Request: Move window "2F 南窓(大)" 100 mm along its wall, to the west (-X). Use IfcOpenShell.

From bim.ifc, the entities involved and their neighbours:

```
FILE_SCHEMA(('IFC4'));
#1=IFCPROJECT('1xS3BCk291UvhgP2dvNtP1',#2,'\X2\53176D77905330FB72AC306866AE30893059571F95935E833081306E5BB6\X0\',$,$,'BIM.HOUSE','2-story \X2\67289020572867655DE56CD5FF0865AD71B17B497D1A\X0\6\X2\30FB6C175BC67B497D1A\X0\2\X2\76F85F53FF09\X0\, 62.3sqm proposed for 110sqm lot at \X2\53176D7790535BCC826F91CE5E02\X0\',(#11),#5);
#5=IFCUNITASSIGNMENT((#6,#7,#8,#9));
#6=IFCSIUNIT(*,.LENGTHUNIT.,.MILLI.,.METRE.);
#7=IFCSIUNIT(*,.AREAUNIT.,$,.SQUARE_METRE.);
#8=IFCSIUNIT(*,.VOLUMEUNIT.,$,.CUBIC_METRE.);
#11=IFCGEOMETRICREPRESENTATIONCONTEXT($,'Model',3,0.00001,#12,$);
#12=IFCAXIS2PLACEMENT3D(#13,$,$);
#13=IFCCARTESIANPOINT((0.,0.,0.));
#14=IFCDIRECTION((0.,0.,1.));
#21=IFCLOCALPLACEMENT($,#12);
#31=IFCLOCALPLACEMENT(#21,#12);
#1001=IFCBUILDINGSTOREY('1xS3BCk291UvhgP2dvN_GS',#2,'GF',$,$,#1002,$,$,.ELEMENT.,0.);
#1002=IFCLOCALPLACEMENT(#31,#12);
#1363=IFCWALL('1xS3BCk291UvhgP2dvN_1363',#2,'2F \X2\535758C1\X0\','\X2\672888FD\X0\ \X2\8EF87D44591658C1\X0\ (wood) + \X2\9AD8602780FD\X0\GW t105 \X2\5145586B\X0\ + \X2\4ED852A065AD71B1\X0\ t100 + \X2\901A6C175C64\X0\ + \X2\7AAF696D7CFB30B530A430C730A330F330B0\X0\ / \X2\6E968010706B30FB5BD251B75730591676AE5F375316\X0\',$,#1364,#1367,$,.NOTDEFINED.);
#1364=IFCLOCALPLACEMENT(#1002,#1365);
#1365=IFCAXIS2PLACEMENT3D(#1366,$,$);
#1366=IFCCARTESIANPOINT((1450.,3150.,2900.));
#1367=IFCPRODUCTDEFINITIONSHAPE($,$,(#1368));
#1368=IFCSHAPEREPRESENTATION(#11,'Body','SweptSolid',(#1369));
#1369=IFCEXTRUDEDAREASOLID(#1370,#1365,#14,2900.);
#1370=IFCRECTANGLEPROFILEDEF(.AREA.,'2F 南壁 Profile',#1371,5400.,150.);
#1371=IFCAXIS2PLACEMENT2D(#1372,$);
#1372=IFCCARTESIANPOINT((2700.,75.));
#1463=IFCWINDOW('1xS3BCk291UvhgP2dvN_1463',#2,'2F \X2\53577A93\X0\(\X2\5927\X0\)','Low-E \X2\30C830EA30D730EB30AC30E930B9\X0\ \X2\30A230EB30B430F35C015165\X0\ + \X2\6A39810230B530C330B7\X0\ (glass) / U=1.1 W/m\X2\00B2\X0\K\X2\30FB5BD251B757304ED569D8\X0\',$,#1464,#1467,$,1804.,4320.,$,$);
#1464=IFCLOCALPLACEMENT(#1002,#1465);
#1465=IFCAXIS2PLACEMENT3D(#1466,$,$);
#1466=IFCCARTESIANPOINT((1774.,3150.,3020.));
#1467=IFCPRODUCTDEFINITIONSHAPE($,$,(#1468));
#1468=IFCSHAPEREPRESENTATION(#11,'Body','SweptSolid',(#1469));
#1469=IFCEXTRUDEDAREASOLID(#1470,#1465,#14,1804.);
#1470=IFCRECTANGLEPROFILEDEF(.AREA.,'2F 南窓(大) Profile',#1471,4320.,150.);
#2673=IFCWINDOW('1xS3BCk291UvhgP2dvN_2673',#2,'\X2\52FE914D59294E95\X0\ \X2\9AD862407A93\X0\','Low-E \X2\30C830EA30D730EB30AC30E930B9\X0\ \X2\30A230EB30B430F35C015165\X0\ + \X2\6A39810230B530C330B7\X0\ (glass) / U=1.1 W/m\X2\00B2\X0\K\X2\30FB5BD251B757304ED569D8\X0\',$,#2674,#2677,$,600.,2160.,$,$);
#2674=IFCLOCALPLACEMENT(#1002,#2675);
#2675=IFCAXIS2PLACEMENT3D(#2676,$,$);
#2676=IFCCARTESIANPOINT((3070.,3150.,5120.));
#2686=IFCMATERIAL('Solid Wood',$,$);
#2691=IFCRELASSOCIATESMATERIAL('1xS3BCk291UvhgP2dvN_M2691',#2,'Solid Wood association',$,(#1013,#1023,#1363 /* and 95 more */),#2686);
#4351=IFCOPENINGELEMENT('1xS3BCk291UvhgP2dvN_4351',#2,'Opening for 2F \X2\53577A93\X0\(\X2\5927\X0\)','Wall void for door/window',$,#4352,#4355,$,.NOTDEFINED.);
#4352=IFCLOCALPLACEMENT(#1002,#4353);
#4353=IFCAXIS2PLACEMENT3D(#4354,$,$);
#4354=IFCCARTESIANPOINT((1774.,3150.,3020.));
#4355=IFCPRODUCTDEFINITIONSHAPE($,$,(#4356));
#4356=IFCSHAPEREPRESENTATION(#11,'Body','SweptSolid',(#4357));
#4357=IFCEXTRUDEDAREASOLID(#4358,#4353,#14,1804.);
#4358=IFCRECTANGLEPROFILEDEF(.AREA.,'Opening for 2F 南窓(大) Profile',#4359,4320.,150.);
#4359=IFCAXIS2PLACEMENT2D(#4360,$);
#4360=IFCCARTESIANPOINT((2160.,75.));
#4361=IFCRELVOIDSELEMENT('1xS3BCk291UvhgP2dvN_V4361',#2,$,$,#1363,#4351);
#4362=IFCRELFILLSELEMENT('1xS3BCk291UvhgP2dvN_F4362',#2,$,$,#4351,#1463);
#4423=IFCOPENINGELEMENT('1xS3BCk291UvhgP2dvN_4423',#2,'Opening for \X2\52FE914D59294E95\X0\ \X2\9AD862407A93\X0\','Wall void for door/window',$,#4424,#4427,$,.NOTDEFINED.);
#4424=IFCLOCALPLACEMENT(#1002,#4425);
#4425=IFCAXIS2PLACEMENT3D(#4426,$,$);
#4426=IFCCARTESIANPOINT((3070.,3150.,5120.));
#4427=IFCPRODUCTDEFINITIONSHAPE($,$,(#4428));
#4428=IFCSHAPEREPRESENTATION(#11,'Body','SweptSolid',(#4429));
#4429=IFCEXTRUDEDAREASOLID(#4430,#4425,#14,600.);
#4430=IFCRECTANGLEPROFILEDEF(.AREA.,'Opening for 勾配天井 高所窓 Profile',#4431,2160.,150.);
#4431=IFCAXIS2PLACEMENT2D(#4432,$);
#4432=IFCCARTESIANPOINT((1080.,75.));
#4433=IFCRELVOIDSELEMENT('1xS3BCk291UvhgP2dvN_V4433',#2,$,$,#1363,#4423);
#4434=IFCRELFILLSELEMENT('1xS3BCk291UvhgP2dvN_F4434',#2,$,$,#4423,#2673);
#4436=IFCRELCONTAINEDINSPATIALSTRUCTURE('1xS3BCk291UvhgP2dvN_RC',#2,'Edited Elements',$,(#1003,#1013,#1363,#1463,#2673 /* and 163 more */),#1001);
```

```python
import ifcopenshell
import ifcopenshell.api.geometry
import ifcopenshell.util.placement
import ifcopenshell.util.unit

model = ifcopenshell.open("bim.ifc")
unit_scale = ifcopenshell.util.unit.calculate_unit_scale(model)

window = model.by_guid("1xS3BCk291UvhgP2dvN_1463")
opening = window.FillsVoids[0].RelatingOpeningElement
wall = opening.VoidsElements[0].RelatingBuildingElement

wall_matrix = ifcopenshell.util.placement.get_local_placement(wall.ObjectPlacement)
shift = wall_matrix[:3, 0] * -0.1 / unit_scale
before = ifcopenshell.util.placement.get_local_placement(window.ObjectPlacement)[:3, 3].copy()

# The window is not placed relative to its opening, so move both.
for product in (opening, window):
    matrix = ifcopenshell.util.placement.get_local_placement(product.ObjectPlacement)
    matrix[:3, 3] += shift
    ifcopenshell.api.geometry.edit_object_placement(model, product=product, matrix=matrix, is_si=False)

after = ifcopenshell.util.placement.get_local_placement(window.ObjectPlacement)[:3, 3]
print("window moved by", (after - before).round(3) + 0.0)

model.write("bim_edited.ifc")
```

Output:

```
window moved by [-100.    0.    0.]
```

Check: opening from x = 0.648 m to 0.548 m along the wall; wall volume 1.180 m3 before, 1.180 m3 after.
